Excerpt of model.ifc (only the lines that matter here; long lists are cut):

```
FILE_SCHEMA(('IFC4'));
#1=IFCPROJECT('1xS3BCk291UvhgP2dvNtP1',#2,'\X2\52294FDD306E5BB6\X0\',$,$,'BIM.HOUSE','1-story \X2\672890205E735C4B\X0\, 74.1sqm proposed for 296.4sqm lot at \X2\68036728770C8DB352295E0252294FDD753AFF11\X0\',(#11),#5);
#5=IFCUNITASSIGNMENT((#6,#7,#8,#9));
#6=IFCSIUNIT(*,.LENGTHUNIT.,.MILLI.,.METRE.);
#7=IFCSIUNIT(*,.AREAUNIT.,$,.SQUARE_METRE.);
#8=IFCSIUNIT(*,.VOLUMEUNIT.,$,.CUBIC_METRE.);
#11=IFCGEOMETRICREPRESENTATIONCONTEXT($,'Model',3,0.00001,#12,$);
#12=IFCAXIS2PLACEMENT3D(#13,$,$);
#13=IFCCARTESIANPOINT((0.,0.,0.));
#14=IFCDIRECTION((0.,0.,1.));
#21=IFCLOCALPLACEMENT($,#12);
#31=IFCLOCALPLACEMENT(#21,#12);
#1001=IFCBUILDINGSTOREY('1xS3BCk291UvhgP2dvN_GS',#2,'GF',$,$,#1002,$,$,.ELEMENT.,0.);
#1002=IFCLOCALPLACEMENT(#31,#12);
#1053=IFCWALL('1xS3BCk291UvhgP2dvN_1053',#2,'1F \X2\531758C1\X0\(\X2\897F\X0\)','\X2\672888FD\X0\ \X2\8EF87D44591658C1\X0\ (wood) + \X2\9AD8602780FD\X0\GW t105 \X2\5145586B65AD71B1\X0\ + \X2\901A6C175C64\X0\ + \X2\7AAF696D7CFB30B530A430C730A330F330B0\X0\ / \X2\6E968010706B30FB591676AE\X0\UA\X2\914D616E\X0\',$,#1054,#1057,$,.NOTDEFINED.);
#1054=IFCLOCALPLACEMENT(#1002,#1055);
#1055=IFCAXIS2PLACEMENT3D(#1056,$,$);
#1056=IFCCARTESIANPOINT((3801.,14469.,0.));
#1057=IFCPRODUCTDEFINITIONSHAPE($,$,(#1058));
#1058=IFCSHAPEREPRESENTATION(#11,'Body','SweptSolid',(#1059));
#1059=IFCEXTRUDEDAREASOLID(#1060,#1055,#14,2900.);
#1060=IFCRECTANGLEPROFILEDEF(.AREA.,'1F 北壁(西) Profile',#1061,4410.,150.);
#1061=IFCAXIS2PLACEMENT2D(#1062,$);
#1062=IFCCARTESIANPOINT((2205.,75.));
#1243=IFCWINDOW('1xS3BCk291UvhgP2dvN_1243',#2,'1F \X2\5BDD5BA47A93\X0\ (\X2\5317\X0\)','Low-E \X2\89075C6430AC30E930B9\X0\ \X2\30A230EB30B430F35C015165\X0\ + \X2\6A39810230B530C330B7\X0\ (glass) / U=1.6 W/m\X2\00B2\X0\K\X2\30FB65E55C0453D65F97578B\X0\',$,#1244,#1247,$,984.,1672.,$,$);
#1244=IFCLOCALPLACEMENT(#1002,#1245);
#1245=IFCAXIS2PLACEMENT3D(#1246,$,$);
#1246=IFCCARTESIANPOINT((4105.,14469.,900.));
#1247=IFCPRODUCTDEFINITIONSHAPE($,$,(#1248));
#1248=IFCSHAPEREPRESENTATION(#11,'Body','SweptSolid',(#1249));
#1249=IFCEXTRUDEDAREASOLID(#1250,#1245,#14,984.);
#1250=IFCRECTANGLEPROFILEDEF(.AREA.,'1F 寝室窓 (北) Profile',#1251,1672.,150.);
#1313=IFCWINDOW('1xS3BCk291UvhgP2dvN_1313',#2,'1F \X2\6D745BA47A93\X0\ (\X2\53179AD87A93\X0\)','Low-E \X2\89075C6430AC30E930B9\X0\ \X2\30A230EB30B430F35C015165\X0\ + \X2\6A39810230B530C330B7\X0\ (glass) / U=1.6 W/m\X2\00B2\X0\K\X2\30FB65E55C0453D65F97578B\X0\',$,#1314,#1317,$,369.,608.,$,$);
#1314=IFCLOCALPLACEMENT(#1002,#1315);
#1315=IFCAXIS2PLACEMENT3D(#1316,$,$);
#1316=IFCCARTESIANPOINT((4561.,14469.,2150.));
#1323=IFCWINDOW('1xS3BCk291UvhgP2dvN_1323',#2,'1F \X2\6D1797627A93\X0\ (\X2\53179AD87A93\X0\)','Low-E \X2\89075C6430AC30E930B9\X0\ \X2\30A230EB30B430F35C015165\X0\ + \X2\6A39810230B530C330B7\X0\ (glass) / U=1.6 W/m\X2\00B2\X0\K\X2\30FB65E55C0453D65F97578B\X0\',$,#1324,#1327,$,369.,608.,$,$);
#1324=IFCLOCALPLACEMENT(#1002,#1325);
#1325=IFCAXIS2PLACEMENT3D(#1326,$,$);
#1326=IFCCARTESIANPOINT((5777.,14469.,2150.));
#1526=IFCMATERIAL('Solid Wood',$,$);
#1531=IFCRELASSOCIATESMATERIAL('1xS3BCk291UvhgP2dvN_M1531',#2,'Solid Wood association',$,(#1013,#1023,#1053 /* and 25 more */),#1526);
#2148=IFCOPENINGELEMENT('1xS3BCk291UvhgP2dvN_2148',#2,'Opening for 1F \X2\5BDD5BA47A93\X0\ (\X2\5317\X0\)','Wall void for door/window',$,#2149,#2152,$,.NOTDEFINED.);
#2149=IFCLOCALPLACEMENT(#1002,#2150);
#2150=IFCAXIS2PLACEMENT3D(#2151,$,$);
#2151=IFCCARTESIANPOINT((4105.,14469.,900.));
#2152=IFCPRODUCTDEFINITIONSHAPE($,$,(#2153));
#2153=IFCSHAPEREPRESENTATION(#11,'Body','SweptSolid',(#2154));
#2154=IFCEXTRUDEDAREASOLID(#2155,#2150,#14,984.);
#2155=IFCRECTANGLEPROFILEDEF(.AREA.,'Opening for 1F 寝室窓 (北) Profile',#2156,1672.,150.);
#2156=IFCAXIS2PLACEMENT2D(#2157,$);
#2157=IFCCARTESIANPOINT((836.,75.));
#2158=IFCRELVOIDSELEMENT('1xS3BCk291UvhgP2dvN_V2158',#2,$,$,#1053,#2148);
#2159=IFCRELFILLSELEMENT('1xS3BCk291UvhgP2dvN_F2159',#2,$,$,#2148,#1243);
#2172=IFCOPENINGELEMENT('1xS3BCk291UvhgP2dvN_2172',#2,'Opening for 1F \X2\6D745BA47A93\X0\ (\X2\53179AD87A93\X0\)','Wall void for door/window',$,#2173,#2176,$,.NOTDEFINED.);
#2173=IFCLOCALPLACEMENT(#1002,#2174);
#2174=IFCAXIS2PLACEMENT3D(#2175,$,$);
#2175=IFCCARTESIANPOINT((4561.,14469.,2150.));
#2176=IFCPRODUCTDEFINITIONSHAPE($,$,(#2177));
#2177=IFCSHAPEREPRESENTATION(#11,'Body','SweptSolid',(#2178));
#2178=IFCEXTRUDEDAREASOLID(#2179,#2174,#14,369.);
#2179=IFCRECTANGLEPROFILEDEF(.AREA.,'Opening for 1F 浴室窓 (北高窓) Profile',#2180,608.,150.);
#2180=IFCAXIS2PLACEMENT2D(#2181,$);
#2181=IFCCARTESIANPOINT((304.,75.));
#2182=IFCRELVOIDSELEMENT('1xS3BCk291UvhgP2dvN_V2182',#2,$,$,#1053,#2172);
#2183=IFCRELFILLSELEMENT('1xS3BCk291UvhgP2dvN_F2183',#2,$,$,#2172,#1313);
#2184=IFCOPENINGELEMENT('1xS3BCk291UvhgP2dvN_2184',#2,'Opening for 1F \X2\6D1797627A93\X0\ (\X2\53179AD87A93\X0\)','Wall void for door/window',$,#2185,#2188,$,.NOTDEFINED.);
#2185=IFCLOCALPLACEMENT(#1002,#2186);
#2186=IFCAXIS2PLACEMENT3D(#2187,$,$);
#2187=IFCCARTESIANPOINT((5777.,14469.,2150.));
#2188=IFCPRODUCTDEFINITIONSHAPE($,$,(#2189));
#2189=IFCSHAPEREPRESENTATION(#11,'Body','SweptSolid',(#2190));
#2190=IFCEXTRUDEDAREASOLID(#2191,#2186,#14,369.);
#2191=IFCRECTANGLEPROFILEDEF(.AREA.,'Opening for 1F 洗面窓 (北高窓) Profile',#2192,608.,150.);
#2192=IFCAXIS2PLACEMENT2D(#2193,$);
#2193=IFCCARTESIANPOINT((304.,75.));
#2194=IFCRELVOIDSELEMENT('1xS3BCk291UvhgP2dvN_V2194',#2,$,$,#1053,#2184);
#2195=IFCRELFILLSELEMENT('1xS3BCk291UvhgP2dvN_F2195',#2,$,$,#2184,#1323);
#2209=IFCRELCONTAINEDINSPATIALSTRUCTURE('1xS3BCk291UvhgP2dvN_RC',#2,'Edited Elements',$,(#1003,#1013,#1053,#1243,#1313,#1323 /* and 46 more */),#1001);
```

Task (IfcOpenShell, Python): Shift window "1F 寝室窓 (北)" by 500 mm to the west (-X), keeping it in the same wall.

```python
import ifcopenshell
import ifcopenshell.api.geometry
import ifcopenshell.util.placement

model = ifcopenshell.open("model.ifc")

window = model.by_guid("1xS3BCk291UvhgP2dvN_1243")
opening = window.FillsVoids[0].RelatingOpeningElement
wall = opening.VoidsElements[0].RelatingBuildingElement

wall_matrix = ifcopenshell.util.placement.get_local_placement(wall.ObjectPlacement)
shift = wall_matrix[:3, 0] * -500.0
before = ifcopenshell.util.placement.get_local_placement(window.ObjectPlacement)[:3, 3].copy()

# The window is not placed relative to its opening, so move both.
for product in (opening, window):
    matrix = ifcopenshell.util.placement.get_local_placement(product.ObjectPlacement)
    matrix[:3, 3] += shift
    ifcopenshell.api.geometry.edit_object_placement(model, product=product, matrix=matrix, is_si=False)

after = ifcopenshell.util.placement.get_local_placement(window.ObjectPlacement)[:3, 3]
print("window moved by", (after - before).round(3) + 0.0)

model.write("model_edited.ifc")
```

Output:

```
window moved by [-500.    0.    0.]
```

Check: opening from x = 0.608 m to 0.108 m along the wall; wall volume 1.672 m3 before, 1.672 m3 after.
